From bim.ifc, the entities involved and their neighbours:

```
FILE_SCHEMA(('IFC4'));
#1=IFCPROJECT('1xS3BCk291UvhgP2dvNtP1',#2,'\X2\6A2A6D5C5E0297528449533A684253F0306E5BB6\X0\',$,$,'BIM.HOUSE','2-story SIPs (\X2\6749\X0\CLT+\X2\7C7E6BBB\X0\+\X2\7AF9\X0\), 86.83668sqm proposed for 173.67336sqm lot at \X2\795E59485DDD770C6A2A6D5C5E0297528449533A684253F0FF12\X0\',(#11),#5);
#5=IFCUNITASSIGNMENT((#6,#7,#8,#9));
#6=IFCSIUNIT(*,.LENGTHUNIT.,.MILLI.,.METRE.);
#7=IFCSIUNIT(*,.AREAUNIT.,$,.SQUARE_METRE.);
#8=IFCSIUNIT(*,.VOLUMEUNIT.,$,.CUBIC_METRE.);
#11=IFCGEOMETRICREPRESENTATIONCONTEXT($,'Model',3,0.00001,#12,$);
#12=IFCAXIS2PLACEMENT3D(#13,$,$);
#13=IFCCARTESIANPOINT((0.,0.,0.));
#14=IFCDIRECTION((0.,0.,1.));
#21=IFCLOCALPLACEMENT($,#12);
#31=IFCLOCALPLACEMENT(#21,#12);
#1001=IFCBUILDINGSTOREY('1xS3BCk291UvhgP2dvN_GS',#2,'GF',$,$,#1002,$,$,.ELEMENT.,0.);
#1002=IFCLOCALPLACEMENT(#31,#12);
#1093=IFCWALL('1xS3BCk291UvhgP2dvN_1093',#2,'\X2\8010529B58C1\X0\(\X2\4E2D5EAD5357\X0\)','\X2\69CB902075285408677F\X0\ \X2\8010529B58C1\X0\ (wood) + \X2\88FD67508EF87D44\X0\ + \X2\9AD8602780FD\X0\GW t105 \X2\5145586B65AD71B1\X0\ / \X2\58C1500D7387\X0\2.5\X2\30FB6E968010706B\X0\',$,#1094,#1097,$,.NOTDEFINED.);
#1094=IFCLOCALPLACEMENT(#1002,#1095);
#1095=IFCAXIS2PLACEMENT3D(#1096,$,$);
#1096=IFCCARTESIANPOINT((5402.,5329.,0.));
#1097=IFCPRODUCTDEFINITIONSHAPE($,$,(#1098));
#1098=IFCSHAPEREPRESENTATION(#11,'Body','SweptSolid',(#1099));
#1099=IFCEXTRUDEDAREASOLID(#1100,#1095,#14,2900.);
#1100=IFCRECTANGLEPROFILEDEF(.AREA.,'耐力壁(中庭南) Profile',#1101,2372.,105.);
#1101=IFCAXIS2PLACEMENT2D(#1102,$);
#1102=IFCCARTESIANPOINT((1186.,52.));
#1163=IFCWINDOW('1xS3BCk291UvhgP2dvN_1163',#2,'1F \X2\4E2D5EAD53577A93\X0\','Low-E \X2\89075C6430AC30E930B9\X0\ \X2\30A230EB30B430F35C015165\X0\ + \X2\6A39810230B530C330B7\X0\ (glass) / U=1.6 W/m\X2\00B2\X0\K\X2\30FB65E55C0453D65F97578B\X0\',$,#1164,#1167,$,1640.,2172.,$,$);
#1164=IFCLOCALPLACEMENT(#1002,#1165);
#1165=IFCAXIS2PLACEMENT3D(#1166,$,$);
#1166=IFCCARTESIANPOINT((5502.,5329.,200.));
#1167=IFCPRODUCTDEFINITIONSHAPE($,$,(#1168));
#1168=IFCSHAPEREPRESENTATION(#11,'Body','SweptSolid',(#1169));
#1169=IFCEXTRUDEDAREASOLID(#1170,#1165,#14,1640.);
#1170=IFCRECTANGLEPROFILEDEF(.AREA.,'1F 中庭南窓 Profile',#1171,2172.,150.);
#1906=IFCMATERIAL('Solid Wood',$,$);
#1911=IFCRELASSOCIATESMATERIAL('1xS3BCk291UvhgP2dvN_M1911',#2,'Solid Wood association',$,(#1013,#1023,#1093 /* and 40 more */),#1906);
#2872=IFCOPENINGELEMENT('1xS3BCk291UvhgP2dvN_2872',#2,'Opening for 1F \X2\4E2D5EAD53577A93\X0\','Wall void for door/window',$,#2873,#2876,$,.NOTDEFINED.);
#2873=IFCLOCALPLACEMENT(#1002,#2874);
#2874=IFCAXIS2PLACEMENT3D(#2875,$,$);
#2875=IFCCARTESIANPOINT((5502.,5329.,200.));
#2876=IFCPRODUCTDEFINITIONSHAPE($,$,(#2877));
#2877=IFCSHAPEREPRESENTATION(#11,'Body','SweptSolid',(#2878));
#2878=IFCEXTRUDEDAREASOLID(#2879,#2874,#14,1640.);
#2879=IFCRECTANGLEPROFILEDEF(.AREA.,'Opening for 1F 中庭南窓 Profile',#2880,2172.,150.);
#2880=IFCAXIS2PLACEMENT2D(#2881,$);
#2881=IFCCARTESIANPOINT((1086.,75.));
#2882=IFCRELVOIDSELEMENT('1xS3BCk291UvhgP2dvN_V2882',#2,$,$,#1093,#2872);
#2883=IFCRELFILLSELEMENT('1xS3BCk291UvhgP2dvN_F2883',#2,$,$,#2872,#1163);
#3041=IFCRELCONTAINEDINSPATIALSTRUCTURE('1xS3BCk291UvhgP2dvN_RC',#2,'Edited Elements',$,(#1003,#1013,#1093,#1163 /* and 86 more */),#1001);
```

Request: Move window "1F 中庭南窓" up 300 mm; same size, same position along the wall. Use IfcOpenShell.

```python
import numpy as np
import ifcopenshell
import ifcopenshell.api.geometry
import ifcopenshell.util.placement
import ifcopenshell.util.unit

model = ifcopenshell.open("bim.ifc")
unit_scale = ifcopenshell.util.unit.calculate_unit_scale(model)

window = model.by_id(1163)
opening = window.FillsVoids[0].RelatingOpeningElement
dz = 300.0

shift = np.array([0.0, 0.0, dz])
# The window is not placed relative to its opening, so move both.
for product in (opening, window):
    matrix = ifcopenshell.util.placement.get_local_placement(product.ObjectPlacement)
    matrix[:3, 3] += shift
    ifcopenshell.api.geometry.edit_object_placement(model, product=product, matrix=matrix, is_si=False)

print(f"moved by {dz * unit_scale:+.3f} m")

model.write("bim_edited.ifc")
```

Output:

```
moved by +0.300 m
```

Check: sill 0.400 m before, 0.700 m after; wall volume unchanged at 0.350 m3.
